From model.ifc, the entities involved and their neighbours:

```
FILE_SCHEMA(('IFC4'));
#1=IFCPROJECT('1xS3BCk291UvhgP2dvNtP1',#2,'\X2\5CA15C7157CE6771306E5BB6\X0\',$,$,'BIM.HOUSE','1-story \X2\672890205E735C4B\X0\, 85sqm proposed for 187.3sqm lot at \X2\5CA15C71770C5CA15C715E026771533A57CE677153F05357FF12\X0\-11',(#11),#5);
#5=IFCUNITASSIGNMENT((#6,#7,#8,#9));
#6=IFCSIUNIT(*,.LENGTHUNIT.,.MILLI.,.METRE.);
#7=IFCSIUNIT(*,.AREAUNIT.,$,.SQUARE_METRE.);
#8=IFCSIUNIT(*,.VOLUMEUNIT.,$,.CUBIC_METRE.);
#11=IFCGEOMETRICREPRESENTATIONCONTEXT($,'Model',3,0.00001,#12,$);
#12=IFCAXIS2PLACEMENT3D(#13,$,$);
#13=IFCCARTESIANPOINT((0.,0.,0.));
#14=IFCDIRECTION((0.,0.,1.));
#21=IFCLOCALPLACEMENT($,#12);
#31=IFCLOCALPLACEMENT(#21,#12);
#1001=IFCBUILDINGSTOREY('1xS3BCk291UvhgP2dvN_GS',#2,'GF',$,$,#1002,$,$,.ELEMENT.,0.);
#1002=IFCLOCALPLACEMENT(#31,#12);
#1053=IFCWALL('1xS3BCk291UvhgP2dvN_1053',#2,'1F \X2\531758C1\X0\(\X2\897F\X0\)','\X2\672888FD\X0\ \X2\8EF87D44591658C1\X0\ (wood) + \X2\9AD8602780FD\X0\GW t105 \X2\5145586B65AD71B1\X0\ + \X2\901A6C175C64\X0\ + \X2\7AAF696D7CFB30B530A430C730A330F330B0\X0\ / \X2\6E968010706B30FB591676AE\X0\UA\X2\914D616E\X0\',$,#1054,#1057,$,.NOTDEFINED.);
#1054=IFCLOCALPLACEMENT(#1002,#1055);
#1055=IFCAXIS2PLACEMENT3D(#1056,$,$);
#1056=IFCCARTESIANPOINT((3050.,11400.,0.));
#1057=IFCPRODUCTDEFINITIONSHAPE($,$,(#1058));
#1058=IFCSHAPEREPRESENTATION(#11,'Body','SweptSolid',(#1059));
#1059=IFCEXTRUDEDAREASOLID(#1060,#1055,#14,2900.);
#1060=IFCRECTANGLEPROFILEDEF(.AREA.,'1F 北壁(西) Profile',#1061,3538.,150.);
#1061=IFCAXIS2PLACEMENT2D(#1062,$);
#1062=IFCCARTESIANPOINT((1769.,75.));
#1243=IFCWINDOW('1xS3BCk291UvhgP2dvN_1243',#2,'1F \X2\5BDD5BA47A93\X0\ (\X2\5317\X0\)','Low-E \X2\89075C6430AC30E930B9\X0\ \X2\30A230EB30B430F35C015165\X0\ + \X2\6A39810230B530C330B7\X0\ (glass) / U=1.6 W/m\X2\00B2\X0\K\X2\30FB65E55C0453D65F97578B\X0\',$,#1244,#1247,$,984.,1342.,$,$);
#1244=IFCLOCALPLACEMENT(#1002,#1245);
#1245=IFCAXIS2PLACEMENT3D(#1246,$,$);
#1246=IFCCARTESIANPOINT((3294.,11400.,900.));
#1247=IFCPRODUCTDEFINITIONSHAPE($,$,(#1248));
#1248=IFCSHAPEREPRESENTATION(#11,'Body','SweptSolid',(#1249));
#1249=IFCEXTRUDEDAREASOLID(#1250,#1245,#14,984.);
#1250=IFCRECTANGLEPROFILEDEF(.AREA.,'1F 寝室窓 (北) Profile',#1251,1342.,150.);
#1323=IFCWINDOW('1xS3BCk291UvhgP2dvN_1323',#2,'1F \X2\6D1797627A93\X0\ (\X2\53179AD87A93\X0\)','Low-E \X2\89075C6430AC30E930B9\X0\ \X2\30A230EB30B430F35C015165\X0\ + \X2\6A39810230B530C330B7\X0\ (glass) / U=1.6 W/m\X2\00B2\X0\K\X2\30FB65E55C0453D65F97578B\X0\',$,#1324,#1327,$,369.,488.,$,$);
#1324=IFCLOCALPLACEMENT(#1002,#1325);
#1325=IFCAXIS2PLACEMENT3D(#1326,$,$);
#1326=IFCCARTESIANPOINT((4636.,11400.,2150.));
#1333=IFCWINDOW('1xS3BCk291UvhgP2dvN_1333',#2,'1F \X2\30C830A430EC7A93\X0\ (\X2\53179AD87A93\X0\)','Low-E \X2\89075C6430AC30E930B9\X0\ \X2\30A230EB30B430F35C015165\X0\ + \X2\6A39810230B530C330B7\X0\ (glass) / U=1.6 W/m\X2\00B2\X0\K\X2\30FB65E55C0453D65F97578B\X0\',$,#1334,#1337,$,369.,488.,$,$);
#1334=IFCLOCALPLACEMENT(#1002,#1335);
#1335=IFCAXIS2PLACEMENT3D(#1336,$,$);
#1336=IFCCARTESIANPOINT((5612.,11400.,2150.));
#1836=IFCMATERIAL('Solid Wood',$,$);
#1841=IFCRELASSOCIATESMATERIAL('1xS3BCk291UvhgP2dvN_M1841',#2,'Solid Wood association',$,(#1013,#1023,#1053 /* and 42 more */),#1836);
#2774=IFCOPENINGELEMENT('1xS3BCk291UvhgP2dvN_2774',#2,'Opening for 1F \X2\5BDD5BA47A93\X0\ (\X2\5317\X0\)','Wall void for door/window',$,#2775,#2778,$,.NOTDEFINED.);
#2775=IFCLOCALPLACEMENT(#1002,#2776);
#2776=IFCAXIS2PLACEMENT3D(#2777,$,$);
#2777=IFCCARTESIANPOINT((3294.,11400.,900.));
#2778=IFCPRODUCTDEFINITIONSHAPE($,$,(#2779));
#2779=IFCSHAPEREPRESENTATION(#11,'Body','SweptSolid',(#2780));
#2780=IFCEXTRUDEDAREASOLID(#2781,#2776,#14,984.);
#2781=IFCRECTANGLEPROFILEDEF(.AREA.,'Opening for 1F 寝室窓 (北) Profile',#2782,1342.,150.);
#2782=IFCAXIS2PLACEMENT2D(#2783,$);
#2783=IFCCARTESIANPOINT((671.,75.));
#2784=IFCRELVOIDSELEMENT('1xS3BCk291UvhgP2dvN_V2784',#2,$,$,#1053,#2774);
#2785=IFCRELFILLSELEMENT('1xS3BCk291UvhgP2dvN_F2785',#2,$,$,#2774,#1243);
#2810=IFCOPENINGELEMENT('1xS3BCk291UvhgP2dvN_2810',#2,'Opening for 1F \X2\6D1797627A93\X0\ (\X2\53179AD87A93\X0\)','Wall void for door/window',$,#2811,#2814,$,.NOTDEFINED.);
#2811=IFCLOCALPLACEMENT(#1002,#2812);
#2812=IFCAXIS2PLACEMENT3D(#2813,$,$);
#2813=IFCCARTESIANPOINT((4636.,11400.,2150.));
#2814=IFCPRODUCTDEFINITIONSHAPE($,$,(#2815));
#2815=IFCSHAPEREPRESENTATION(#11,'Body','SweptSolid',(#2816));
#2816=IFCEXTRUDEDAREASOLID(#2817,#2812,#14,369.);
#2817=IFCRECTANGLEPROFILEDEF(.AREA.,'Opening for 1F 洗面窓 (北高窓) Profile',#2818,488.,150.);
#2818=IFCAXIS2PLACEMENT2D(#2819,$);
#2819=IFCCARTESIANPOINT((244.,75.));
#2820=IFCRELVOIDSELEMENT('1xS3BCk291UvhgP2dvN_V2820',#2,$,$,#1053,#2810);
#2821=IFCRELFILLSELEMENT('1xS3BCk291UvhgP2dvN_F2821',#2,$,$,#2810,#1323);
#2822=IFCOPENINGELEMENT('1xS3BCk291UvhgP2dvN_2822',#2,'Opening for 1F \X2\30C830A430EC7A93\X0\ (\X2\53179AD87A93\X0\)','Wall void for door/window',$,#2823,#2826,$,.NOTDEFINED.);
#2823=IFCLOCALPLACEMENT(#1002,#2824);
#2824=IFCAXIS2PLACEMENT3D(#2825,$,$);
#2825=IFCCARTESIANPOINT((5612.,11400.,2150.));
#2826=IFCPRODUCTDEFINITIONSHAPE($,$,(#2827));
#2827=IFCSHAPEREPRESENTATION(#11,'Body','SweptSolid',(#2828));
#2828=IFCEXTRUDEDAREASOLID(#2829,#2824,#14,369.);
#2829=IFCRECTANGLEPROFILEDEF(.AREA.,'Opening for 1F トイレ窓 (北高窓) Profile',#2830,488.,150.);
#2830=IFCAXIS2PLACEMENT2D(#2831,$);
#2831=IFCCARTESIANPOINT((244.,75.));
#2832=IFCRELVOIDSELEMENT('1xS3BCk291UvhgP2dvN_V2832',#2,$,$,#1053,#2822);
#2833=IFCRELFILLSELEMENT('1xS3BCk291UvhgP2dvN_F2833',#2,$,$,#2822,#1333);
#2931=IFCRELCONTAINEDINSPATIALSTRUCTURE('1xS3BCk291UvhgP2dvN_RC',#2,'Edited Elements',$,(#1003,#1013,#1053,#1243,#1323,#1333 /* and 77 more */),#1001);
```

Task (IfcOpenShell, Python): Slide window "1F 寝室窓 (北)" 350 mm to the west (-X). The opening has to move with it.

```python
import ifcopenshell
import ifcopenshell.api.geometry
import ifcopenshell.util.placement

model = ifcopenshell.open("model.ifc")

window = model.by_id(1243)
opening = window.FillsVoids[0].RelatingOpeningElement
wall = opening.VoidsElements[0].RelatingBuildingElement

wall_matrix = ifcopenshell.util.placement.get_local_placement(wall.ObjectPlacement)
shift = wall_matrix[:3, 0] * -350.0
before = ifcopenshell.util.placement.get_local_placement(window.ObjectPlacement)[:3, 3].copy()

# The window is not placed relative to its opening, so move both.
for product in (opening, window):
    matrix = ifcopenshell.util.placement.get_local_placement(product.ObjectPlacement)
    matrix[:3, 3] += shift
    ifcopenshell.api.geometry.edit_object_placement(model, product=product, matrix=matrix, is_si=False)

after = ifcopenshell.util.placement.get_local_placement(window.ObjectPlacement)[:3, 3]
print("window moved by", (after - before).round(3) + 0.0)

model.write("model_edited.ifc")
```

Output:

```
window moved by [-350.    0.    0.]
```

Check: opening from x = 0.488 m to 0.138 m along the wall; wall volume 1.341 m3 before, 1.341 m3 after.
